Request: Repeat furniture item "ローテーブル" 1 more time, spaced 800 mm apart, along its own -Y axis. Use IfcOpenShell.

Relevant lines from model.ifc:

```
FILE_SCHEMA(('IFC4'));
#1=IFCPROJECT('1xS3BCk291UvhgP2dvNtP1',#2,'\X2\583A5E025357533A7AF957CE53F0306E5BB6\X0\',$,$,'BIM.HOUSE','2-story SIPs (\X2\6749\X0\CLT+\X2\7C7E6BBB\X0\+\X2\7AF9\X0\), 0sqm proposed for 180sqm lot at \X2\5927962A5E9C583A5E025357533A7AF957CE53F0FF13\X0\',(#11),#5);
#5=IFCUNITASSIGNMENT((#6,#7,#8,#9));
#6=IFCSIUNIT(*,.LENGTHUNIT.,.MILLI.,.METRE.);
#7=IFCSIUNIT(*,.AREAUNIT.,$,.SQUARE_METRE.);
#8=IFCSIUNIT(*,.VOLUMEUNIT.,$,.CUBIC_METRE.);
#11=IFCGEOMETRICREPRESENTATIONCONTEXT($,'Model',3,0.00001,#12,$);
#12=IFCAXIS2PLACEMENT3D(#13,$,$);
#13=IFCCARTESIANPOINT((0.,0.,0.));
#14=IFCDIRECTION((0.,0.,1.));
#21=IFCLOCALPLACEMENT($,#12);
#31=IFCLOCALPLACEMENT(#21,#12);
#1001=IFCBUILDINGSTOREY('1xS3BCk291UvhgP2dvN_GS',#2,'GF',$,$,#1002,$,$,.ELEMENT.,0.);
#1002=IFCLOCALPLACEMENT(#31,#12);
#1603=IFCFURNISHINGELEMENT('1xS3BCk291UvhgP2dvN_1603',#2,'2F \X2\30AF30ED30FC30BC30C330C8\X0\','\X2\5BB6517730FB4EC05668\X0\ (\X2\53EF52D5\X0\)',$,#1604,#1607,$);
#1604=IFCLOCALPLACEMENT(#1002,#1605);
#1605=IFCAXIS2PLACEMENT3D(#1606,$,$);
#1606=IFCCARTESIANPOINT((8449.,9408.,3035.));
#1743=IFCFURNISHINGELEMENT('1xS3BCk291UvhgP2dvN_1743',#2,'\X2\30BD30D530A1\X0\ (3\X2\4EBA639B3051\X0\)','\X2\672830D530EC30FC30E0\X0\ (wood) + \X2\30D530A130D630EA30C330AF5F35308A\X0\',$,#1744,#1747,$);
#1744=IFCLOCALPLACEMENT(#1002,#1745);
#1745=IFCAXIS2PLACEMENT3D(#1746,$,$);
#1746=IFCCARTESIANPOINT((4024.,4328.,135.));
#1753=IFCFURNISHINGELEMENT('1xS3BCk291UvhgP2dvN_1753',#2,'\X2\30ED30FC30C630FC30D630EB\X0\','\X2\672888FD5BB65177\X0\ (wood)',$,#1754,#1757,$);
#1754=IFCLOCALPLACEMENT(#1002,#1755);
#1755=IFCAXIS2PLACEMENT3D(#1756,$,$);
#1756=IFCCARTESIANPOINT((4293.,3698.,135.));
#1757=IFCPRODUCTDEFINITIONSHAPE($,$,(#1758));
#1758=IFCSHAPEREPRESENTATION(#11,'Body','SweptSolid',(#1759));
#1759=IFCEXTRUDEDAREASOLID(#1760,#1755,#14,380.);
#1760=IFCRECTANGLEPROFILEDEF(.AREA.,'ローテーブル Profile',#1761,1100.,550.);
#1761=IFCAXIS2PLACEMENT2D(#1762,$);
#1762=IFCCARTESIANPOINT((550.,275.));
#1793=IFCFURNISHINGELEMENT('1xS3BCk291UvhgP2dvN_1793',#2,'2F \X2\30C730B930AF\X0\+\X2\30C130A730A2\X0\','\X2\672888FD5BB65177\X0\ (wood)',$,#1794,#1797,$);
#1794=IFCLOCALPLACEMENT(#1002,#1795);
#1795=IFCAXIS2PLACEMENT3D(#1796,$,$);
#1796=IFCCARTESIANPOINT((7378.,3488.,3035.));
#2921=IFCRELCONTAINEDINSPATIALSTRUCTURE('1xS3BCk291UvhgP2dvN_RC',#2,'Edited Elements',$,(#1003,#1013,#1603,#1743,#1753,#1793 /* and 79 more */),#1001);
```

```python
import ifcopenshell
import ifcopenshell.api.geometry
import ifcopenshell.api.root
import ifcopenshell.util.element
import ifcopenshell.util.placement
import ifcopenshell.util.unit

model = ifcopenshell.open("model.ifc")
unit_scale = ifcopenshell.util.unit.calculate_unit_scale(model)


def reuse_history(source, copy):
    """copy_class also copies each property set's owner history, people and application; keep the originals."""
    for rel in copy.IsDefinedBy:
        if rel.is_a("IfcRelDefinesByProperties") and (history := rel.RelatingPropertyDefinition.OwnerHistory):
            rel.RelatingPropertyDefinition.OwnerHistory = source.OwnerHistory
            ifcopenshell.util.element.remove_deep2(model, history)


source = model.by_guid("1xS3BCk291UvhgP2dvN_1753")
base = ifcopenshell.util.placement.get_local_placement(source.ObjectPlacement)
step = -base[:3, 1] * 0.8 / unit_scale

for i in range(1, 2):
    copy = ifcopenshell.api.root.copy_class(model, product=source)
    copy.Representation = ifcopenshell.util.element.copy_deep(
        model, source.Representation, exclude=["IfcGeometricRepresentationContext", "IfcRepresentationMap"]
    )
    reuse_history(source, copy)
    matrix = base.copy()
    matrix[:3, 3] += i * step
    print("added at", matrix[:3, 3].round(3) + 0.0)
    ifcopenshell.api.geometry.edit_object_placement(model, product=copy, matrix=matrix, is_si=False)

model.write("model_rev.ifc")
```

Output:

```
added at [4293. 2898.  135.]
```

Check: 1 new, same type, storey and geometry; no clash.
